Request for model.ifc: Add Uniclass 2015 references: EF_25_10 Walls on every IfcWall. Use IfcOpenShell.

First a look at what the model holds.

```python
import ifcopenshell

model = ifcopenshell.open("model.ifc")
print(model.schema)
print("classifications:", [c.Name for c in model.by_type("IfcClassification")])
for ifc_class in ("IfcDoor", "IfcRoof", "IfcStair", "IfcWall", "IfcWindow"):
    print(ifc_class, len(model.by_type(ifc_class)))
```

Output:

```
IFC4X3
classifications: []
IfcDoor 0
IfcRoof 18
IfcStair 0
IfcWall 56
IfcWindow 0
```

```python
import ifcopenshell
import ifcopenshell.api.classification

model = ifcopenshell.open("model.ifc")

system = ifcopenshell.api.classification.add_classification(model, classification="Uniclass 2015")

codes = {
    "IfcWall": ("EF_25_10", "Walls"),
}
for ifc_class, (code, name) in codes.items():
    products = model.by_type(ifc_class)
    ifcopenshell.api.classification.add_reference(
        model, products=products, classification=system, identification=code, name=name
    )
    print(code, len(products))

model.write("model_v2.ifc")
```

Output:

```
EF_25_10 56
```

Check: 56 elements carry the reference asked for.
